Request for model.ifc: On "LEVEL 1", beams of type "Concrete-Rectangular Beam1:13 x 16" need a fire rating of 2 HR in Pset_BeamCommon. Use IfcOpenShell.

First a look at what the model holds.

```python
import ifcopenshell
import ifcopenshell.util.element

model = ifcopenshell.open("model.ifc")
print(model.schema)
storey = next(s for s in model.by_type("IfcBuildingStorey") if s.Name == "LEVEL 1")
beams = [e for e in ifcopenshell.util.element.get_decomposition(storey) if e.is_a("IfcBeam")]
seen = {}
for e in beams:
    element_type = ifcopenshell.util.element.get_type(e)
    key = (element_type.Name if element_type != e and element_type else None, ifcopenshell.util.element.get_pset(e, "Pset_BeamCommon", "FireRating"))
    seen[key] = seen.get(key, 0) + 1
for (name, value), count in sorted(seen.items(), key=str):
    print(count, "x", name, "|", value)
```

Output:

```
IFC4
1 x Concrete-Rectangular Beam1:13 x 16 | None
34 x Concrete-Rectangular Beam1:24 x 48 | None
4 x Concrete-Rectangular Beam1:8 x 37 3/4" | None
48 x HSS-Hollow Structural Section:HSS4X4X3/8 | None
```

```python
import ifcopenshell
import ifcopenshell.api.pset
import ifcopenshell.util.element

model = ifcopenshell.open("model.ifc")

storey = next(s for s in model.by_type("IfcBuildingStorey") if s.Name == "LEVEL 1")
beams = [e for e in ifcopenshell.util.element.get_decomposition(storey) if e.is_a("IfcBeam")]

count = 0
for e in beams:
    element_type = ifcopenshell.util.element.get_type(e)
    if element_type in (None, e) or element_type.Name != "Concrete-Rectangular Beam1:13 x 16":
        continue
    # add_pset returns the element's existing set when there is one.
    pset = ifcopenshell.api.pset.add_pset(model, product=e, name="Pset_BeamCommon")
    ifcopenshell.api.pset.edit_pset(model, pset=pset, properties={"FireRating": "2 HR"})
    count += 1

print(count, "beams updated")

model.write("model_updated.ifc")
```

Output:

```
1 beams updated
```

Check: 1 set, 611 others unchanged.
